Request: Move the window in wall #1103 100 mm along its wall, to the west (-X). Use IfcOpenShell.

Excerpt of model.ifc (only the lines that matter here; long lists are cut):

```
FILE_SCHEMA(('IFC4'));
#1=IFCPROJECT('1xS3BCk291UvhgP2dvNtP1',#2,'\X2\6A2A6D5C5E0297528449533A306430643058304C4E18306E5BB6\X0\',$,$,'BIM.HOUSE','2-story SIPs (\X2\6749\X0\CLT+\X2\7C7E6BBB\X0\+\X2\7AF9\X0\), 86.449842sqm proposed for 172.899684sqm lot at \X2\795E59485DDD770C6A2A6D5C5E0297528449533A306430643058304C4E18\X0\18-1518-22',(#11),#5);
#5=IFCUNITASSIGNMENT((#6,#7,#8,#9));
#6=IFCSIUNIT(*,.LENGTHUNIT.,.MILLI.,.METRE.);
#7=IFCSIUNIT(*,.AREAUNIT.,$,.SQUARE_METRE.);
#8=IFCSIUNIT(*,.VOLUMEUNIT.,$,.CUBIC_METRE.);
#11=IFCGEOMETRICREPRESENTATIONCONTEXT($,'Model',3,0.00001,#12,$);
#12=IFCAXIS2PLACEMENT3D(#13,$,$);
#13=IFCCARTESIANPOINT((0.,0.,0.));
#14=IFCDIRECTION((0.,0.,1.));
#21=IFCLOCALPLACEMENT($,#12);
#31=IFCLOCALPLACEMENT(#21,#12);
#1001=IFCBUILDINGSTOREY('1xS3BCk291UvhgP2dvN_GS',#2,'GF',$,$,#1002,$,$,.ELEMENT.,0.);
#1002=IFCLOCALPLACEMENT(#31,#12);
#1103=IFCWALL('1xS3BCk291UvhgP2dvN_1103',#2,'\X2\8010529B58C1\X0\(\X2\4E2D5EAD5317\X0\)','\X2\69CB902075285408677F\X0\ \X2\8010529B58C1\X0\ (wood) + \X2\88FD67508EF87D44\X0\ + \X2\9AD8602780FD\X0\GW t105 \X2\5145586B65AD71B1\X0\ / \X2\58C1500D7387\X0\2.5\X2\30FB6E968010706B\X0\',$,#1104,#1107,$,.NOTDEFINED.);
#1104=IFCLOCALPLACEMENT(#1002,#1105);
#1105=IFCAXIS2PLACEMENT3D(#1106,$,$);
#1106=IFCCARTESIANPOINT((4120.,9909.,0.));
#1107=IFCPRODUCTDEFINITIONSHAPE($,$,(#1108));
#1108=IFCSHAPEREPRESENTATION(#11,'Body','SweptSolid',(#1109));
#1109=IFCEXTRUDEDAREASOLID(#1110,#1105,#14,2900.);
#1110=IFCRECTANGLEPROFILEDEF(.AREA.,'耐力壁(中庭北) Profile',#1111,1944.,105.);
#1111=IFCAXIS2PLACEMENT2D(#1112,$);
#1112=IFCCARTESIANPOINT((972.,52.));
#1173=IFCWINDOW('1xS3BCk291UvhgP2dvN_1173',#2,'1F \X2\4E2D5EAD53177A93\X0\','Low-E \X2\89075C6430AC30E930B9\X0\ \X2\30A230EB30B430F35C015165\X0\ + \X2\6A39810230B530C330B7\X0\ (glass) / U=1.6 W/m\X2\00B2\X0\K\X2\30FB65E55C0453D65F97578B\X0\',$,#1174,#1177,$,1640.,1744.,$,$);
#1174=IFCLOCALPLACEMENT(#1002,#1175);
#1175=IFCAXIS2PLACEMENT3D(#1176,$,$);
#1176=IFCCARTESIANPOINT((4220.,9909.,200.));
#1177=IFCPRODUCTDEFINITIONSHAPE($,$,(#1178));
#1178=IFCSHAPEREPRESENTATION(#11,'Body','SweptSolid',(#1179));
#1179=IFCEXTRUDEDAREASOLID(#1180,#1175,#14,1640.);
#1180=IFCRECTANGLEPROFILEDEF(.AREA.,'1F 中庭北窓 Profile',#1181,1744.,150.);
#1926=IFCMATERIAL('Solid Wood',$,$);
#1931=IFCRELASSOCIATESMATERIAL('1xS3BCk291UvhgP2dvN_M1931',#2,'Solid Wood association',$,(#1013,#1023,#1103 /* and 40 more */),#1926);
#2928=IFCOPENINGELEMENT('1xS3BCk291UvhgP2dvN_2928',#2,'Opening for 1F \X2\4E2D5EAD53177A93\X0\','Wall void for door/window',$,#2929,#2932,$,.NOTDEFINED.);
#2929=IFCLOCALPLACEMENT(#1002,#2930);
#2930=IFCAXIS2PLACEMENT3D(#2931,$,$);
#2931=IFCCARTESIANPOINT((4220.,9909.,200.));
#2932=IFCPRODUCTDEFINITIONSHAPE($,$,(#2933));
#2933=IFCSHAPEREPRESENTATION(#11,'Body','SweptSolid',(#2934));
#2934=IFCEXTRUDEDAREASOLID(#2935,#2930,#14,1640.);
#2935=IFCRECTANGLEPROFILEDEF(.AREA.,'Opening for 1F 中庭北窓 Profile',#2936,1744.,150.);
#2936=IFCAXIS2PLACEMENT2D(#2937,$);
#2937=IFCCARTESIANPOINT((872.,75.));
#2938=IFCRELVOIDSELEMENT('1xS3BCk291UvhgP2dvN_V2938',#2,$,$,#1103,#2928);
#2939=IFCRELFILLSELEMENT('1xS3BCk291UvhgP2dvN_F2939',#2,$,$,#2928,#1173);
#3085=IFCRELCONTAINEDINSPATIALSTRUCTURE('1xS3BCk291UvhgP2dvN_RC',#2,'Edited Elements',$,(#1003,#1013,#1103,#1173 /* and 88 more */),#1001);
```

```python
import ifcopenshell
import ifcopenshell.api.geometry
import ifcopenshell.util.placement
import ifcopenshell.util.unit

model = ifcopenshell.open("model.ifc")
unit_scale = ifcopenshell.util.unit.calculate_unit_scale(model)

window = model.by_id(1173)
opening = window.FillsVoids[0].RelatingOpeningElement
wall = opening.VoidsElements[0].RelatingBuildingElement

wall_matrix = ifcopenshell.util.placement.get_local_placement(wall.ObjectPlacement)
shift = wall_matrix[:3, 0] * -0.1 / unit_scale
before = ifcopenshell.util.placement.get_local_placement(window.ObjectPlacement)[:3, 3].copy()

# The window is not placed relative to its opening, so move both.
for product in (opening, window):
    matrix = ifcopenshell.util.placement.get_local_placement(product.ObjectPlacement)
    matrix[:3, 3] += shift
    ifcopenshell.api.geometry.edit_object_placement(model, product=product, matrix=matrix, is_si=False)

after = ifcopenshell.util.placement.get_local_placement(window.ObjectPlacement)[:3, 3]
print("window moved by", (after - before).round(3) + 0.0)

model.write("model_edited.ifc")
```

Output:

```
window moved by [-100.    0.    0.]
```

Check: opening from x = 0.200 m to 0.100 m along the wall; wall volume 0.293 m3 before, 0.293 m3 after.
